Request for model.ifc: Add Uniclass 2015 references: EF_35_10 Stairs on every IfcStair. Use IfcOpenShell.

First a look at what the model holds.

```python
import ifcopenshell

model = ifcopenshell.open("model.ifc")
print(model.schema)
print("classifications:", [c.Name for c in model.by_type("IfcClassification")])
for ifc_class in ("IfcDoor", "IfcRoof", "IfcStair", "IfcWall", "IfcWindow"):
    print(ifc_class, len(model.by_type(ifc_class)))
```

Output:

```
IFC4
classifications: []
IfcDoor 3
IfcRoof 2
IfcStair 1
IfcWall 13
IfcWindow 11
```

```python
import ifcopenshell
import ifcopenshell.api.classification

model = ifcopenshell.open("model.ifc")

system = ifcopenshell.api.classification.add_classification(model, classification="Uniclass 2015")

codes = {
    "IfcStair": ("EF_35_10", "Stairs"),
}
for ifc_class, (code, name) in codes.items():
    products = model.by_type(ifc_class)
    ifcopenshell.api.classification.add_reference(
        model, products=products, classification=system, identification=code, name=name
    )
    print(code, len(products))

model.write("model_v2.ifc")
```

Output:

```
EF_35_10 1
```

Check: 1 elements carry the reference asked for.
